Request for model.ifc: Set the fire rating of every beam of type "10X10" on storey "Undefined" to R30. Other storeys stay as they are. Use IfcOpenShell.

First a look at what the model holds.

```python
import ifcopenshell
import ifcopenshell.util.element

model = ifcopenshell.open("model.ifc")
print(model.schema)
storey = next(s for s in model.by_type("IfcBuildingStorey") if s.Name == "Undefined")
beams = [e for e in ifcopenshell.util.element.get_decomposition(storey) if e.is_a("IfcBeam")]
seen = {}
for e in beams:
    element_type = ifcopenshell.util.element.get_type(e)
    key = (element_type.Name if element_type != e and element_type else None, ifcopenshell.util.element.get_pset(e, "Pset_BeamCommon", "FireRating"))
    seen[key] = seen.get(key, 0) + 1
for (name, value), count in sorted(seen.items(), key=str):
    print(count, "x", name, "|", value)
```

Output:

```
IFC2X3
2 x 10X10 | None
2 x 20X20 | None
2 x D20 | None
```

```python
import ifcopenshell
import ifcopenshell.api.pset
import ifcopenshell.util.element

model = ifcopenshell.open("model.ifc")

storey = next(s for s in model.by_type("IfcBuildingStorey") if s.Name == "Undefined")
beams = [e for e in ifcopenshell.util.element.get_decomposition(storey) if e.is_a("IfcBeam")]

count = 0
for e in beams:
    element_type = ifcopenshell.util.element.get_type(e)
    if element_type in (None, e) or element_type.Name != "10X10":
        continue
    found = ifcopenshell.util.element.get_pset(e, "Pset_BeamCommon", should_inherit=False)
    if found:
        pset = model.by_id(found["id"])
        if len(ifcopenshell.util.element.get_elements_by_pset(pset)) > 1:
            pset = ifcopenshell.api.pset.unshare_pset(model, products=[e], pset=pset)[0]
    else:
        pset = ifcopenshell.api.pset.add_pset(model, product=e, name="Pset_BeamCommon")
    ifcopenshell.api.pset.edit_pset(model, pset=pset, properties={"FireRating": "R30"})
    count += 1

print(count, "beams updated")

model.write("model_updated.ifc")
```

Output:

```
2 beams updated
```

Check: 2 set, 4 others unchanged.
